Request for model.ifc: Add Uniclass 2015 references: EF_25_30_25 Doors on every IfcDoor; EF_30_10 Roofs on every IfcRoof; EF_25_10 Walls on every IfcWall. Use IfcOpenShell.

First a look at what the model holds.

```python
import ifcopenshell

model = ifcopenshell.open("model.ifc")
print(model.schema)
print("classifications:", [c.Name for c in model.by_type("IfcClassification")])
for ifc_class in ("IfcDoor", "IfcRoof", "IfcStair", "IfcWall", "IfcWindow"):
    print(ifc_class, len(model.by_type(ifc_class)))
```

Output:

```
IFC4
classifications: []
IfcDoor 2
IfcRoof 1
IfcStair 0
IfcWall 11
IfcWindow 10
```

```python
import ifcopenshell
import ifcopenshell.api.classification

model = ifcopenshell.open("model.ifc")

system = ifcopenshell.api.classification.add_classification(model, classification="Uniclass 2015")

codes = {
    "IfcDoor": ("EF_25_30_25", "Doors"),
    "IfcRoof": ("EF_30_10", "Roofs"),
    "IfcWall": ("EF_25_10", "Walls"),
}
for ifc_class, (code, name) in codes.items():
    products = model.by_type(ifc_class)
    ifcopenshell.api.classification.add_reference(
        model, products=products, classification=system, identification=code, name=name
    )
    print(code, len(products))

model.write("model_updated.ifc")
```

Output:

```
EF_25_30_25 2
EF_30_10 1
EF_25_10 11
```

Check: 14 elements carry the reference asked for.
